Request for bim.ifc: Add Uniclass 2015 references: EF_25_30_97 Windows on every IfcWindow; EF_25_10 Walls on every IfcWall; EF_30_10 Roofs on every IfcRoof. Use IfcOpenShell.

First a look at what the model holds.

```python
import ifcopenshell

model = ifcopenshell.open("bim.ifc")
print(model.schema)
print("classifications:", [c.Name for c in model.by_type("IfcClassification")])
for ifc_class in ("IfcDoor", "IfcRoof", "IfcStair", "IfcWall", "IfcWindow"):
    print(ifc_class, len(model.by_type(ifc_class)))
```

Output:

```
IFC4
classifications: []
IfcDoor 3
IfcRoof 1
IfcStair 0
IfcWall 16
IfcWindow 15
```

```python
import ifcopenshell
import ifcopenshell.api.classification

model = ifcopenshell.open("bim.ifc")

system = ifcopenshell.api.classification.add_classification(model, classification="Uniclass 2015")

codes = {
    "IfcWindow": ("EF_25_30_97", "Windows"),
    "IfcWall": ("EF_25_10", "Walls"),
    "IfcRoof": ("EF_30_10", "Roofs"),
}
for ifc_class, (code, name) in codes.items():
    products = model.by_type(ifc_class)
    ifcopenshell.api.classification.add_reference(
        model, products=products, classification=system, identification=code, name=name
    )
    print(code, len(products))

model.write("bim_v2.ifc")
```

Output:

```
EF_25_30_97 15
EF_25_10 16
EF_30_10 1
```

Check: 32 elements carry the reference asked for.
